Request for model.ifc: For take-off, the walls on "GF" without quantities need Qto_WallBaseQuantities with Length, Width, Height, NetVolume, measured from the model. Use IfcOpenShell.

First a look at what the model holds.

```python
import ifcopenshell
import ifcopenshell.util.element
import ifcopenshell.util.unit

model = ifcopenshell.open("model.ifc")
print(model.schema)
for unit_type in ("LENGTHUNIT", "AREAUNIT", "VOLUMEUNIT"):
    print(unit_type, ifcopenshell.util.unit.calculate_unit_scale(model, unit_type))
storey = next(s for s in model.by_type("IfcBuildingStorey") if s.Name == "GF")
walls = [e for e in ifcopenshell.util.element.get_decomposition(storey) if e.is_a("IfcWall")]
for e in sorted(walls, key=lambda e: e.id()):
    print(e.id(), e.is_a(), e.Name, list(ifcopenshell.util.element.get_psets(e, qtos_only=True)), sep=" | ")
```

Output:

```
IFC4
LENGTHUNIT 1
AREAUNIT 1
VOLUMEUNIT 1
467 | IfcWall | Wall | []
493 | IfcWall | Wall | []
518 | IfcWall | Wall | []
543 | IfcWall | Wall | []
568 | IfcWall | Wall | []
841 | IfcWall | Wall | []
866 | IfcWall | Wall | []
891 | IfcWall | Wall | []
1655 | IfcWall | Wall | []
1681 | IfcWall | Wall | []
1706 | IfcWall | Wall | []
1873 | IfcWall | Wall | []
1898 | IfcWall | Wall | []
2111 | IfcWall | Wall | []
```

```python
import ifcopenshell
import ifcopenshell.api.pset
import ifcopenshell.geom
import ifcopenshell.util.element
import ifcopenshell.util.shape
import ifcopenshell.util.unit

model = ifcopenshell.open("model.ifc")
unit_scale = ifcopenshell.util.unit.calculate_unit_scale(model)
volume_scale = ifcopenshell.util.unit.calculate_unit_scale(model, "VOLUMEUNIT")
settings = ifcopenshell.geom.settings()

storey = next(s for s in model.by_type("IfcBuildingStorey") if s.Name == "GF")
walls = [e for e in ifcopenshell.util.element.get_decomposition(storey) if e.is_a("IfcWall")]

for e in sorted(walls, key=lambda e: e.id()):
    if ifcopenshell.util.element.get_psets(e, qtos_only=True, should_inherit=False):
        continue
    # Geometry comes back in metres, in the element's own axes.
    shape = ifcopenshell.geom.create_shape(settings, e)
    values = {
        "Length": ifcopenshell.util.shape.get_x(shape.geometry) / unit_scale,
        "Width": ifcopenshell.util.shape.get_y(shape.geometry) / unit_scale,
        "Height": ifcopenshell.util.shape.get_z(shape.geometry) / unit_scale,
        "NetVolume": ifcopenshell.util.shape.get_volume(shape.geometry) / volume_scale,
    }
    qto = ifcopenshell.api.pset.add_qto(model, product=e, name="Qto_WallBaseQuantities")
    ifcopenshell.api.pset.edit_qto(model, qto=qto, properties=values)
    print(e.id(), {k: round(v, 3) for k, v in values.items()})

model.write("model_rev.ifc")
```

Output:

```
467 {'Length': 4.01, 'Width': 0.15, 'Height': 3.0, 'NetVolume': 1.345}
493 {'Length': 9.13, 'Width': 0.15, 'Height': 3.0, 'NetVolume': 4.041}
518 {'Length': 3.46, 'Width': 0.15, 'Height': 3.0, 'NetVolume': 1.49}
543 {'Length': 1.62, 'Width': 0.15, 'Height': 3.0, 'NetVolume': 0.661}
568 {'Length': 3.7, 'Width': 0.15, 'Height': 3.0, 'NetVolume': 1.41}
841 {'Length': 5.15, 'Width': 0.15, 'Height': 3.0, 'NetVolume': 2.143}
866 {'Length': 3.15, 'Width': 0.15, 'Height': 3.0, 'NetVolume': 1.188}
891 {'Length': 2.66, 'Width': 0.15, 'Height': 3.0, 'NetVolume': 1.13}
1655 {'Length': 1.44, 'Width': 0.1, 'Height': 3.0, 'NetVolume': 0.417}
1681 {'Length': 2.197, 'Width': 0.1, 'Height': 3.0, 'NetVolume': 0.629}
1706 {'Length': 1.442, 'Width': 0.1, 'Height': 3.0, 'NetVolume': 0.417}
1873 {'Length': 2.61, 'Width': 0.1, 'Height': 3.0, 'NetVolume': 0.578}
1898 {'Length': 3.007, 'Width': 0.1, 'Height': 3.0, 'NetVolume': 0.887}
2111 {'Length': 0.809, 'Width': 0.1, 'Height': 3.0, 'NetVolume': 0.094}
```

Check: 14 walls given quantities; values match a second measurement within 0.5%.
